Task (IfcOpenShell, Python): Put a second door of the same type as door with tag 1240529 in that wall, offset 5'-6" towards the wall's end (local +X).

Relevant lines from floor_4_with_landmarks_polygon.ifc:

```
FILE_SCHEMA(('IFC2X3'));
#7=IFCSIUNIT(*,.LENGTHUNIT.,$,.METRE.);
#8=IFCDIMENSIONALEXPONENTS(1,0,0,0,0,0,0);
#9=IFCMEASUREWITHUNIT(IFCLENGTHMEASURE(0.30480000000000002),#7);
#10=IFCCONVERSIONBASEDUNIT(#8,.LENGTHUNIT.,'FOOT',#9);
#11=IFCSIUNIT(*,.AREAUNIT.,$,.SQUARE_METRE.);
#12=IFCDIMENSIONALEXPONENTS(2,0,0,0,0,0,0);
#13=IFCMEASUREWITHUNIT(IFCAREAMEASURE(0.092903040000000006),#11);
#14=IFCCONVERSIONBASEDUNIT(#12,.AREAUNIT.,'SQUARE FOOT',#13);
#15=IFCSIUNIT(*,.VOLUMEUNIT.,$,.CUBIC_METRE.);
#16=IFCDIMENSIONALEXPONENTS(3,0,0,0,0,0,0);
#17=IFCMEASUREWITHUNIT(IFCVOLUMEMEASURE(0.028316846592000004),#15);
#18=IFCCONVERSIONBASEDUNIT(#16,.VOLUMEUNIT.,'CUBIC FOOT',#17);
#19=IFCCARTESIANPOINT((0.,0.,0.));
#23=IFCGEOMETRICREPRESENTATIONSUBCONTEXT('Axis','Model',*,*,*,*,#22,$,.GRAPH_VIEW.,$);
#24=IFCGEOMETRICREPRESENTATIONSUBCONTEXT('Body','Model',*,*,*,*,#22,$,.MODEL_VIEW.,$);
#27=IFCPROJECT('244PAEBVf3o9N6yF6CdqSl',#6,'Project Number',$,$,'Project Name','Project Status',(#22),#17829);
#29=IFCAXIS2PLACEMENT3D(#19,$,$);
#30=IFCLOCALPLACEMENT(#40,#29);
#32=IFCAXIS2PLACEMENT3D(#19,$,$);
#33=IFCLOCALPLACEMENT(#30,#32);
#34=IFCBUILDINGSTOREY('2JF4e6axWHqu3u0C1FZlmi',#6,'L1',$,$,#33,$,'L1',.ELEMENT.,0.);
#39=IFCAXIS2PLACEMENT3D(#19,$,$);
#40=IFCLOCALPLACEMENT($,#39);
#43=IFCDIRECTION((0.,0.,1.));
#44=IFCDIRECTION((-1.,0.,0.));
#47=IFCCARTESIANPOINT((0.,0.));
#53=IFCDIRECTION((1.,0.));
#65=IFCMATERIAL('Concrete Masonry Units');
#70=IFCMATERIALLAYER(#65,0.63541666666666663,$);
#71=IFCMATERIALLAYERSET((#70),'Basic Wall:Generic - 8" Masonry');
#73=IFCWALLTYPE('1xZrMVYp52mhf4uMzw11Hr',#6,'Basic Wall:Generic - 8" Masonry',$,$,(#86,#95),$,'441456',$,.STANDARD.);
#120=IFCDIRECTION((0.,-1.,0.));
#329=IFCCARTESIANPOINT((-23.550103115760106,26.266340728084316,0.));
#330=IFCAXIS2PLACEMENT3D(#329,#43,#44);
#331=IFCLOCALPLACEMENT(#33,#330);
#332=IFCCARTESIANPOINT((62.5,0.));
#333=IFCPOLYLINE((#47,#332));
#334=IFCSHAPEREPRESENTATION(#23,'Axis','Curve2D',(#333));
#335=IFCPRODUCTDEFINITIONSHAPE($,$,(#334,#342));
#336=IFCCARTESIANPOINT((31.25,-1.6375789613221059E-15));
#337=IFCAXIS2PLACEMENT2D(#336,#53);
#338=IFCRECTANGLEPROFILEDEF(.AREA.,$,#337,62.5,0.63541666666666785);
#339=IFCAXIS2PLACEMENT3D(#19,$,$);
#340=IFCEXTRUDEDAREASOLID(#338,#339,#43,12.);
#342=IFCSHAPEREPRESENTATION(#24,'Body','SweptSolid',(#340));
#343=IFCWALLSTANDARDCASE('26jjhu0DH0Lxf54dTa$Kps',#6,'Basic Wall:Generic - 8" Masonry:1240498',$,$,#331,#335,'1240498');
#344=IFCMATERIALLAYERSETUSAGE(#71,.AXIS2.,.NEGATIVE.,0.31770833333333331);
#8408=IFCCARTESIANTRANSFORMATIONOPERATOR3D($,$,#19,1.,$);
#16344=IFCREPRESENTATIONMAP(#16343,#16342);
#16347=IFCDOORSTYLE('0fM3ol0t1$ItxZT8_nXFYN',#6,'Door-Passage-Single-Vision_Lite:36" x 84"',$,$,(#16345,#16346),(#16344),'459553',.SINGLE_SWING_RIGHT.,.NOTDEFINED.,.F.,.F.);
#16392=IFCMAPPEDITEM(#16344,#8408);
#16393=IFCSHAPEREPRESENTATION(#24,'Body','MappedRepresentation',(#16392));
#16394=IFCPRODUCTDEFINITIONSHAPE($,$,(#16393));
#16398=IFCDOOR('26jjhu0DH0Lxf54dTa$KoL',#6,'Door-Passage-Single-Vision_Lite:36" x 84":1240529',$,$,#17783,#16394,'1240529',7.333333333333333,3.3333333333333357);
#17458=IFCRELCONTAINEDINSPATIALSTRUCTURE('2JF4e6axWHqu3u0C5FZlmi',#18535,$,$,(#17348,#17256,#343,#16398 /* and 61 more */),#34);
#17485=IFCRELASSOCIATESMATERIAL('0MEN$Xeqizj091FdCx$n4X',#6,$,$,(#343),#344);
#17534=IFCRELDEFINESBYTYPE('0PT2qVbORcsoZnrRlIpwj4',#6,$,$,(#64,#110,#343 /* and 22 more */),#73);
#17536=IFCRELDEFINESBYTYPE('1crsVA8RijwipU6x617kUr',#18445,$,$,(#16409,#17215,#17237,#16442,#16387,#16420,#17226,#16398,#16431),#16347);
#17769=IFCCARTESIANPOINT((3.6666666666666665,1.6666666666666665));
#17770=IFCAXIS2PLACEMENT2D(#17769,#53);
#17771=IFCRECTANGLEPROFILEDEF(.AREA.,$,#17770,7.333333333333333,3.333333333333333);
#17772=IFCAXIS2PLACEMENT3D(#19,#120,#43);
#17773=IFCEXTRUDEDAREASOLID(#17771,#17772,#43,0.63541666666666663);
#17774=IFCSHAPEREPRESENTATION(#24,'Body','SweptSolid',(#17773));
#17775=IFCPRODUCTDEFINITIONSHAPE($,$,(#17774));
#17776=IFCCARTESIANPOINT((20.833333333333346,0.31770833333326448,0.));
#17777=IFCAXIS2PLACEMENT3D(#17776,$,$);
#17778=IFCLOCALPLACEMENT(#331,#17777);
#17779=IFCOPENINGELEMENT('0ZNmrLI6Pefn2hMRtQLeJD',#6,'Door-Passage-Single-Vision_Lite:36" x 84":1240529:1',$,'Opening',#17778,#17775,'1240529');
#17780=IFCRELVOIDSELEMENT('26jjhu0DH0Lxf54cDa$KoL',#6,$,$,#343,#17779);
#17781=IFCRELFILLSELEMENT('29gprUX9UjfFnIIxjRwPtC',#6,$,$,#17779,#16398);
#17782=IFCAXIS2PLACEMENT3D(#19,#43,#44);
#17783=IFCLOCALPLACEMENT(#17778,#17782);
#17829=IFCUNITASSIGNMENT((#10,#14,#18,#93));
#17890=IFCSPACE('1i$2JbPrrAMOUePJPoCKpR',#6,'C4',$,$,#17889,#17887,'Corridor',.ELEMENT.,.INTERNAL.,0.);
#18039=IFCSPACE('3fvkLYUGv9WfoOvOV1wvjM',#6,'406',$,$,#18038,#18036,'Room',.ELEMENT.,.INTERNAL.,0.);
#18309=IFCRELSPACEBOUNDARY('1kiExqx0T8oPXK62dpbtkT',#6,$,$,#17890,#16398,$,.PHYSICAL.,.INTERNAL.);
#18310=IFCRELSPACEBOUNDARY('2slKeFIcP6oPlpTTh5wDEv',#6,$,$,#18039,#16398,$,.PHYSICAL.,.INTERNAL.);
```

```python
import ifcopenshell
import ifcopenshell.api.feature
import ifcopenshell.api.geometry
import ifcopenshell.api.root
import ifcopenshell.geom
import ifcopenshell.util.element
import ifcopenshell.util.placement
import ifcopenshell.util.shape
import ifcopenshell.util.unit

model = ifcopenshell.open("floor_4_with_landmarks_polygon.ifc")
unit_scale = ifcopenshell.util.unit.calculate_unit_scale(model)
settings = ifcopenshell.geom.settings()


def volume(element):
    """Net volume in cubic metres, openings subtracted."""
    shape = ifcopenshell.geom.create_shape(settings, element)
    return ifcopenshell.util.shape.get_volume(shape.geometry)


def reuse_history(source, copy):
    """copy_class also copies each property set's owner history, people and application; keep the originals."""
    for rel in copy.IsDefinedBy:
        if rel.is_a("IfcRelDefinesByProperties") and (history := rel.RelatingPropertyDefinition.OwnerHistory):
            rel.RelatingPropertyDefinition.OwnerHistory = source.OwnerHistory
            ifcopenshell.util.element.remove_deep2(model, history)


door = model.by_guid("26jjhu0DH0Lxf54dTa$KoL")
opening = door.FillsVoids[0].RelatingOpeningElement
wall = opening.VoidsElements[0].RelatingBuildingElement
before = volume(wall)
shift = ifcopenshell.util.placement.get_local_placement(wall.ObjectPlacement)[:3, 0] * 66 * 0.0254 / unit_scale

# copy_class copies the void relationship, type, container and properties, but no geometry.
new_opening = ifcopenshell.api.root.copy_class(model, product=opening)
new_opening.Representation = ifcopenshell.util.element.copy_deep(
    model, opening.Representation, exclude=["IfcGeometricRepresentationContext", "IfcRepresentationMap"]
)
new_opening.Name = 'Door-Passage-Single-Vision_Lite:36" x 84"'
new_opening.Tag = None
new_door = ifcopenshell.api.root.copy_class(model, product=door)
new_door.Representation = ifcopenshell.util.element.copy_deep(
    model, door.Representation, exclude=["IfcGeometricRepresentationContext", "IfcRepresentationMap"]
)
new_door.Name = 'Door-Passage-Single-Vision_Lite:36" x 84"'
new_door.Tag = None
reuse_history(door, new_door)
fills = ifcopenshell.api.feature.add_filling(model, opening=new_opening, element=new_door)
fills.OwnerHistory = new_door.OwnerHistory  # required in IFC2X3

for old, new in ((opening, new_opening), (door, new_door)):
    matrix = ifcopenshell.util.placement.get_local_placement(old.ObjectPlacement)
    matrix[:3, 3] += shift
    ifcopenshell.api.geometry.edit_object_placement(model, product=new, matrix=matrix, is_si=False)

after = volume(wall)

print(f"wall volume {before:.3f} -> {after:.3f} m3")

model.write("floor_4_with_landmarks_polygon_updated.ifc")
```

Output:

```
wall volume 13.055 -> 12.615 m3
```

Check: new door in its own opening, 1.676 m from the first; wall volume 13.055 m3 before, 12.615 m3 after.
